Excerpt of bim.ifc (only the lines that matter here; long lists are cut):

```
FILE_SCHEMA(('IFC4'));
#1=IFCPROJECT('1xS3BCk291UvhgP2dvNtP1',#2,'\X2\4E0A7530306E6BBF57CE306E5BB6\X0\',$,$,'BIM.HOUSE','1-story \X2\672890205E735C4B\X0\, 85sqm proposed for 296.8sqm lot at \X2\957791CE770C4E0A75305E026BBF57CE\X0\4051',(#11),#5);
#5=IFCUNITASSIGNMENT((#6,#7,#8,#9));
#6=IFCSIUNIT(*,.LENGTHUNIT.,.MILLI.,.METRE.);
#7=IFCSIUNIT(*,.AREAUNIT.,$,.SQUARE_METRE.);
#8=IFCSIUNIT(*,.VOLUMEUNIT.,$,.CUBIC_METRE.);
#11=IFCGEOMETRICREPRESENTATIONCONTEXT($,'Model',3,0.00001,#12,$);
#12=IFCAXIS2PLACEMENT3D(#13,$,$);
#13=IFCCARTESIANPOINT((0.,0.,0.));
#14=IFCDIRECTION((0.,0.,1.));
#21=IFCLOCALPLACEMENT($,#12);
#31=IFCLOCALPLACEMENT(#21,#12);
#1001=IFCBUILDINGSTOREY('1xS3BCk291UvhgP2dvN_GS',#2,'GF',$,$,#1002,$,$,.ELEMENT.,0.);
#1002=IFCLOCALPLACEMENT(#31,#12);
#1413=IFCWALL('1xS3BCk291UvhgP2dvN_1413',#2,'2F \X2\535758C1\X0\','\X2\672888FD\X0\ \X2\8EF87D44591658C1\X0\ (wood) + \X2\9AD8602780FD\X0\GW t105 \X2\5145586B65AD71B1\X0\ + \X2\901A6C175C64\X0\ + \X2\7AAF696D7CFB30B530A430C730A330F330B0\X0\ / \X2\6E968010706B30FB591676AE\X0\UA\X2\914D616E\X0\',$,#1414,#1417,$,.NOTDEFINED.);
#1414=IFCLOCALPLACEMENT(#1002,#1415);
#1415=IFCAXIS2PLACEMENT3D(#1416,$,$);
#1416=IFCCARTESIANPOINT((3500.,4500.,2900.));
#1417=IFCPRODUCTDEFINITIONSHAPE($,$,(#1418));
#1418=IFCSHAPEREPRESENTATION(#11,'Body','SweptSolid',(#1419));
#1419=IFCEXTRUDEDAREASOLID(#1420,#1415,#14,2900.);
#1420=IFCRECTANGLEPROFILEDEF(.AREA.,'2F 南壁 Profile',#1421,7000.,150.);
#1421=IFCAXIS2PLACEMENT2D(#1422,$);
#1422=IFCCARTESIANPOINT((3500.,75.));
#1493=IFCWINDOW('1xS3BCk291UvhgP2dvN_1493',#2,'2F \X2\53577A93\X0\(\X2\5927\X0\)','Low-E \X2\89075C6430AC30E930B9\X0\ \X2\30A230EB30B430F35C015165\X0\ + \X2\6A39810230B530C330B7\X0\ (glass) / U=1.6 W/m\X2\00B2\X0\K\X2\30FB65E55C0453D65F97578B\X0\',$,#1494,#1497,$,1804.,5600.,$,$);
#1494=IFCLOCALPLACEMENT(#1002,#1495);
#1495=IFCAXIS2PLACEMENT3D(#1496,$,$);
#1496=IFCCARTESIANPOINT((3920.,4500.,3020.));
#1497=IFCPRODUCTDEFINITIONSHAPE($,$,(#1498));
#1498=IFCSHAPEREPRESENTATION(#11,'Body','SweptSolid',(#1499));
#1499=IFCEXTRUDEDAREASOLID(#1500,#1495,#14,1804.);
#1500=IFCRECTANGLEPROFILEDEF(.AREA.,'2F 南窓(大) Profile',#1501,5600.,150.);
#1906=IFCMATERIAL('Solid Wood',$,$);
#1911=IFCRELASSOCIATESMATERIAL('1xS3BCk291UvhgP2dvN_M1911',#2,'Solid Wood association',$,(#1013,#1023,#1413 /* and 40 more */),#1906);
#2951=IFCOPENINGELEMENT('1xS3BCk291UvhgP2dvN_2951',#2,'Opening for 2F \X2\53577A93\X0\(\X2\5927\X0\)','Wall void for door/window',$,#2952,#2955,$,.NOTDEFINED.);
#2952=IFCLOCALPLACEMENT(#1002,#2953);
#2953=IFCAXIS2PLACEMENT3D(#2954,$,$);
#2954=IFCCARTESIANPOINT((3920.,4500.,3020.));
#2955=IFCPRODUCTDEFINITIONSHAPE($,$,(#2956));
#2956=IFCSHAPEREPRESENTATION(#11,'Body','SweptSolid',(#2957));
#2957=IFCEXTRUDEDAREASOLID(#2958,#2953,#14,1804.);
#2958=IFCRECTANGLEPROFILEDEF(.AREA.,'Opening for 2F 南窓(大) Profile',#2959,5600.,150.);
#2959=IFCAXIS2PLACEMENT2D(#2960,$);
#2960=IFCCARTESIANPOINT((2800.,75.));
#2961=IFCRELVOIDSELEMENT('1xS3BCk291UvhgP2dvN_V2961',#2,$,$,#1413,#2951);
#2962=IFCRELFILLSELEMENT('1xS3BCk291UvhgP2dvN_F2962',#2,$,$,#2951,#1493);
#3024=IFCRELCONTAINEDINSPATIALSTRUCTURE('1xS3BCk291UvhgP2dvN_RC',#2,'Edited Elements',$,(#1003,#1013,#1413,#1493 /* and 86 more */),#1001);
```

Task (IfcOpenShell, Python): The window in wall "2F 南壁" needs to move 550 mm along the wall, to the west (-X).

```python
import ifcopenshell
import ifcopenshell.api.geometry
import ifcopenshell.util.placement
import ifcopenshell.util.unit

model = ifcopenshell.open("bim.ifc")
unit_scale = ifcopenshell.util.unit.calculate_unit_scale(model)

window = model.by_guid("1xS3BCk291UvhgP2dvN_1493")
opening = window.FillsVoids[0].RelatingOpeningElement
wall = opening.VoidsElements[0].RelatingBuildingElement

wall_matrix = ifcopenshell.util.placement.get_local_placement(wall.ObjectPlacement)
shift = wall_matrix[:3, 0] * -0.55 / unit_scale
before = ifcopenshell.util.placement.get_local_placement(window.ObjectPlacement)[:3, 3].copy()

# The window is not placed relative to its opening, so move both.
for product in (opening, window):
    matrix = ifcopenshell.util.placement.get_local_placement(product.ObjectPlacement)
    matrix[:3, 3] += shift
    ifcopenshell.api.geometry.edit_object_placement(model, product=product, matrix=matrix, is_si=False)

after = ifcopenshell.util.placement.get_local_placement(window.ObjectPlacement)[:3, 3]
print("window moved by", (after - before).round(3) + 0.0)

model.write("bim_rev.ifc")
```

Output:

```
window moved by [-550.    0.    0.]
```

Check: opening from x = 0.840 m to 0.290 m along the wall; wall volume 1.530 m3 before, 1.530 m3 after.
